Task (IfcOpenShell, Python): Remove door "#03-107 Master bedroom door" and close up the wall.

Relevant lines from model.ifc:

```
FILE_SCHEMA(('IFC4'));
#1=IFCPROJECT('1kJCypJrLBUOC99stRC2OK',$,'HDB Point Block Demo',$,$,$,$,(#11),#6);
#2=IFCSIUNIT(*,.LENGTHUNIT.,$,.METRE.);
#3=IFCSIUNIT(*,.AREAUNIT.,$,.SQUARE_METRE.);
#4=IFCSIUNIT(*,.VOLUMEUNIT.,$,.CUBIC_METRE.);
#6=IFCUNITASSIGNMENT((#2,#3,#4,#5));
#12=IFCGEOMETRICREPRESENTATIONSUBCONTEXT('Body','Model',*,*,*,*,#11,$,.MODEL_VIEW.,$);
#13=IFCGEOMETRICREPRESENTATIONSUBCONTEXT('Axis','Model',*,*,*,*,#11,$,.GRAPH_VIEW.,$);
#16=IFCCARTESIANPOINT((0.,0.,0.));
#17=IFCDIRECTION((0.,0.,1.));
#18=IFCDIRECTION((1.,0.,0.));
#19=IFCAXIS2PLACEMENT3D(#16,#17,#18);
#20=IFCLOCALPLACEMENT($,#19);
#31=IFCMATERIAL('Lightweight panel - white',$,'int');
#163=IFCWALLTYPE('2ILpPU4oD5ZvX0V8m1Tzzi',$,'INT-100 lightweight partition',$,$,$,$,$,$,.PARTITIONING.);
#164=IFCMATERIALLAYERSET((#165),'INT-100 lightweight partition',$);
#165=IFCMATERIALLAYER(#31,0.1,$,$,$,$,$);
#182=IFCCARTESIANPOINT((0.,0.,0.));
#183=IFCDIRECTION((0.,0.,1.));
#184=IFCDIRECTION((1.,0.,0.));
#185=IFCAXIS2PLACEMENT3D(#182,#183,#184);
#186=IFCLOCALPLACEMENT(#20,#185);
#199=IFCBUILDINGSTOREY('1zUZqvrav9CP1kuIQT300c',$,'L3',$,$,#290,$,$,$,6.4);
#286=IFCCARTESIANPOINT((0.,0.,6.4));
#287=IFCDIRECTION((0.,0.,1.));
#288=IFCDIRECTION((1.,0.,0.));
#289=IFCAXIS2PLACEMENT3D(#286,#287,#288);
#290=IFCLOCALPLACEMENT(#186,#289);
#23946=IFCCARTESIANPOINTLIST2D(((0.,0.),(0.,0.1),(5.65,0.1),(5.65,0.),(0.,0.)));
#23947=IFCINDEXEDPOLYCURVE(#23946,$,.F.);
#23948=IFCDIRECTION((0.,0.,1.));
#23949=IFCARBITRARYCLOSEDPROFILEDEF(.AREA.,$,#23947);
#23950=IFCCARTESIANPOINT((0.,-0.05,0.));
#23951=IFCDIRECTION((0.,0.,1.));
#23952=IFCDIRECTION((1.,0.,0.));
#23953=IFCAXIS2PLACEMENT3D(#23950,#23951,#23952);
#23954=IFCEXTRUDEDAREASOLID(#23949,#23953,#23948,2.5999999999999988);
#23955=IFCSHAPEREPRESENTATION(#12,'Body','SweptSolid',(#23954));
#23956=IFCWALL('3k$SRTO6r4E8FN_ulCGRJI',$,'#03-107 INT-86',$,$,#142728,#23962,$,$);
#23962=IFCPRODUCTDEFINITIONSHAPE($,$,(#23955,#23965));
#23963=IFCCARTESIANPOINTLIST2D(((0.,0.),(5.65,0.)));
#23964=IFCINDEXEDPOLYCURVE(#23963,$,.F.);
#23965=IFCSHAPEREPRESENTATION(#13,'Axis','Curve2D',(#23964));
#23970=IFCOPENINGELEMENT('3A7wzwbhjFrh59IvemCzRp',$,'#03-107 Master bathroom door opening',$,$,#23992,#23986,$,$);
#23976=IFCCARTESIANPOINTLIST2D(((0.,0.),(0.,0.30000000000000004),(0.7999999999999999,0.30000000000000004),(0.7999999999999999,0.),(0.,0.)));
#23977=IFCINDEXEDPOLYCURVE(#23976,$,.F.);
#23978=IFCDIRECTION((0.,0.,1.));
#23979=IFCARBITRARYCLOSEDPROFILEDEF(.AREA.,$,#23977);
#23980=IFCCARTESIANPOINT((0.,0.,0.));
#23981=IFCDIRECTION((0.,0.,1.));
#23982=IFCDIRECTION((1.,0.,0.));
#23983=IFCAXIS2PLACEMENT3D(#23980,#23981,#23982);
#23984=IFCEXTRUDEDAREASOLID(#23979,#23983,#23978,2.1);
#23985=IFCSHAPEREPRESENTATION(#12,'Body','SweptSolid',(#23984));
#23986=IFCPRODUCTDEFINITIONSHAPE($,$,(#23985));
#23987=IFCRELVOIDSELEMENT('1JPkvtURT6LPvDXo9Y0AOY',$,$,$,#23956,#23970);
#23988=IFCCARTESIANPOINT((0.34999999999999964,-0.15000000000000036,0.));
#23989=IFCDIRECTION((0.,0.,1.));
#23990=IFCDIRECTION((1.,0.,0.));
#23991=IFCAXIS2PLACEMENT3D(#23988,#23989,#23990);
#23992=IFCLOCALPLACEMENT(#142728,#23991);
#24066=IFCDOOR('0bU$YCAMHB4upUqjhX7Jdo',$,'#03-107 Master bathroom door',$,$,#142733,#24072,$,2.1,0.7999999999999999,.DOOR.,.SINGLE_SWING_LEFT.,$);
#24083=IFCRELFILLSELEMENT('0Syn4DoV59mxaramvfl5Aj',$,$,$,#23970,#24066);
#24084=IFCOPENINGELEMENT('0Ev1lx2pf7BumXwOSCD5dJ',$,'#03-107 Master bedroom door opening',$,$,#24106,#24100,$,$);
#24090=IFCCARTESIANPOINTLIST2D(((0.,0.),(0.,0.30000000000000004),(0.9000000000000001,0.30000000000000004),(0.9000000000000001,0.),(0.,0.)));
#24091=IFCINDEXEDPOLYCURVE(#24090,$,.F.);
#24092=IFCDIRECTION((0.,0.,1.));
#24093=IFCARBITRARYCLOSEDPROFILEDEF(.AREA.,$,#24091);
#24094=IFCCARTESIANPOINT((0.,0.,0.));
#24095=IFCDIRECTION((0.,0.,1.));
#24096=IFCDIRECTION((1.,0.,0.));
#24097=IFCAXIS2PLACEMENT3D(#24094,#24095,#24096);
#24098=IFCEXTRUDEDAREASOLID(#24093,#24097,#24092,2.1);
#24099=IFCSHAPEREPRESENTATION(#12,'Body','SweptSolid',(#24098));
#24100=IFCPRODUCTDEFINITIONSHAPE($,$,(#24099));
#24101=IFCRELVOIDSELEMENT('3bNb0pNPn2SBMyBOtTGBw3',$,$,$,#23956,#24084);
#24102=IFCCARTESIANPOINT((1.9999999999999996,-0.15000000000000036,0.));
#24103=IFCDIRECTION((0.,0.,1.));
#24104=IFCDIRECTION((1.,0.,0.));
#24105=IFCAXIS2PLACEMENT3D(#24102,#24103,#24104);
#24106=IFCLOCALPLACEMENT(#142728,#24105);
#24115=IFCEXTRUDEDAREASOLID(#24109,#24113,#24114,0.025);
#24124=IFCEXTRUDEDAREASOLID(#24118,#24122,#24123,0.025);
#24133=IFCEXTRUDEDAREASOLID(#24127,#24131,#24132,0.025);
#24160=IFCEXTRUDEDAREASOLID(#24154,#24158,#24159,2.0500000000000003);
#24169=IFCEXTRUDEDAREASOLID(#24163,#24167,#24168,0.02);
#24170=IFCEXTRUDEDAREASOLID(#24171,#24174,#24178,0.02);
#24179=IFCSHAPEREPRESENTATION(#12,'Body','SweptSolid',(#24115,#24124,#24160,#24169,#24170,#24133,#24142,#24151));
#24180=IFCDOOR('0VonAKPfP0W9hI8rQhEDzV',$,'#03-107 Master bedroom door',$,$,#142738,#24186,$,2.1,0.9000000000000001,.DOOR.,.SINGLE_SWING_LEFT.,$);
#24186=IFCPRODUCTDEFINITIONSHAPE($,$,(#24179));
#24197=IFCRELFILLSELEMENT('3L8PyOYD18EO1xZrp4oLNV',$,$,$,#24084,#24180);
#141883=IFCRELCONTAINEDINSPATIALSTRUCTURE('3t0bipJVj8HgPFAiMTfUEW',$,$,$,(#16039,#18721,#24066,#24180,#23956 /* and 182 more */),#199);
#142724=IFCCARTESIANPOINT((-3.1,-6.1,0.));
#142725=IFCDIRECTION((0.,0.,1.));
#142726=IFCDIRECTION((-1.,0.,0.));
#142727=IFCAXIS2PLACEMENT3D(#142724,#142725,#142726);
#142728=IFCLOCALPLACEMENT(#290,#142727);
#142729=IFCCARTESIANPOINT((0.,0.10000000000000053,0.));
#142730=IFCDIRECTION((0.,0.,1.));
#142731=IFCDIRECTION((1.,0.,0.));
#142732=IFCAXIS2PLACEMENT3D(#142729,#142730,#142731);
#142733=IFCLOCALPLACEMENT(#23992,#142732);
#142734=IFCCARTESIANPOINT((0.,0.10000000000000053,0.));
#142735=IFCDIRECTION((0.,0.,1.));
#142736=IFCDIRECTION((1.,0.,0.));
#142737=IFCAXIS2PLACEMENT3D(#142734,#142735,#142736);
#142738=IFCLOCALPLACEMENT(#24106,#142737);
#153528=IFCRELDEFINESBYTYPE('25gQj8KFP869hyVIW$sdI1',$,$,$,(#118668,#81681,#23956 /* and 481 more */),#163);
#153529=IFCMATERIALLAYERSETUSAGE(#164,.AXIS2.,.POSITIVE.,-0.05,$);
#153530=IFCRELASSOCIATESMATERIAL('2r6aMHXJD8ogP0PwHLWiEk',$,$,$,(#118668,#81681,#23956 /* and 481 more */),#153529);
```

```python
import ifcopenshell
import ifcopenshell.api.feature
import ifcopenshell.api.root
import ifcopenshell.geom
import ifcopenshell.util.shape

model = ifcopenshell.open("model.ifc")
settings = ifcopenshell.geom.settings()


def volume(element):
    """Net volume in cubic metres, openings subtracted."""
    shape = ifcopenshell.geom.create_shape(settings, element)
    return ifcopenshell.util.shape.get_volume(shape.geometry)


door = model.by_guid("0VonAKPfP0W9hI8rQhEDzV")
opening = door.FillsVoids[0].RelatingOpeningElement
wall = opening.VoidsElements[0].RelatingBuildingElement
before = volume(wall)

ifcopenshell.api.root.remove_product(model, product=door)
ifcopenshell.api.feature.remove_feature(model, feature=opening)

after = volume(wall)

print(f"wall volume {before:.3f} -> {after:.3f} m3")

model.write("model_updated.ifc")
```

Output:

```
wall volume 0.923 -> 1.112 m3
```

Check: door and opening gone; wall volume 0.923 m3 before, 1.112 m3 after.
